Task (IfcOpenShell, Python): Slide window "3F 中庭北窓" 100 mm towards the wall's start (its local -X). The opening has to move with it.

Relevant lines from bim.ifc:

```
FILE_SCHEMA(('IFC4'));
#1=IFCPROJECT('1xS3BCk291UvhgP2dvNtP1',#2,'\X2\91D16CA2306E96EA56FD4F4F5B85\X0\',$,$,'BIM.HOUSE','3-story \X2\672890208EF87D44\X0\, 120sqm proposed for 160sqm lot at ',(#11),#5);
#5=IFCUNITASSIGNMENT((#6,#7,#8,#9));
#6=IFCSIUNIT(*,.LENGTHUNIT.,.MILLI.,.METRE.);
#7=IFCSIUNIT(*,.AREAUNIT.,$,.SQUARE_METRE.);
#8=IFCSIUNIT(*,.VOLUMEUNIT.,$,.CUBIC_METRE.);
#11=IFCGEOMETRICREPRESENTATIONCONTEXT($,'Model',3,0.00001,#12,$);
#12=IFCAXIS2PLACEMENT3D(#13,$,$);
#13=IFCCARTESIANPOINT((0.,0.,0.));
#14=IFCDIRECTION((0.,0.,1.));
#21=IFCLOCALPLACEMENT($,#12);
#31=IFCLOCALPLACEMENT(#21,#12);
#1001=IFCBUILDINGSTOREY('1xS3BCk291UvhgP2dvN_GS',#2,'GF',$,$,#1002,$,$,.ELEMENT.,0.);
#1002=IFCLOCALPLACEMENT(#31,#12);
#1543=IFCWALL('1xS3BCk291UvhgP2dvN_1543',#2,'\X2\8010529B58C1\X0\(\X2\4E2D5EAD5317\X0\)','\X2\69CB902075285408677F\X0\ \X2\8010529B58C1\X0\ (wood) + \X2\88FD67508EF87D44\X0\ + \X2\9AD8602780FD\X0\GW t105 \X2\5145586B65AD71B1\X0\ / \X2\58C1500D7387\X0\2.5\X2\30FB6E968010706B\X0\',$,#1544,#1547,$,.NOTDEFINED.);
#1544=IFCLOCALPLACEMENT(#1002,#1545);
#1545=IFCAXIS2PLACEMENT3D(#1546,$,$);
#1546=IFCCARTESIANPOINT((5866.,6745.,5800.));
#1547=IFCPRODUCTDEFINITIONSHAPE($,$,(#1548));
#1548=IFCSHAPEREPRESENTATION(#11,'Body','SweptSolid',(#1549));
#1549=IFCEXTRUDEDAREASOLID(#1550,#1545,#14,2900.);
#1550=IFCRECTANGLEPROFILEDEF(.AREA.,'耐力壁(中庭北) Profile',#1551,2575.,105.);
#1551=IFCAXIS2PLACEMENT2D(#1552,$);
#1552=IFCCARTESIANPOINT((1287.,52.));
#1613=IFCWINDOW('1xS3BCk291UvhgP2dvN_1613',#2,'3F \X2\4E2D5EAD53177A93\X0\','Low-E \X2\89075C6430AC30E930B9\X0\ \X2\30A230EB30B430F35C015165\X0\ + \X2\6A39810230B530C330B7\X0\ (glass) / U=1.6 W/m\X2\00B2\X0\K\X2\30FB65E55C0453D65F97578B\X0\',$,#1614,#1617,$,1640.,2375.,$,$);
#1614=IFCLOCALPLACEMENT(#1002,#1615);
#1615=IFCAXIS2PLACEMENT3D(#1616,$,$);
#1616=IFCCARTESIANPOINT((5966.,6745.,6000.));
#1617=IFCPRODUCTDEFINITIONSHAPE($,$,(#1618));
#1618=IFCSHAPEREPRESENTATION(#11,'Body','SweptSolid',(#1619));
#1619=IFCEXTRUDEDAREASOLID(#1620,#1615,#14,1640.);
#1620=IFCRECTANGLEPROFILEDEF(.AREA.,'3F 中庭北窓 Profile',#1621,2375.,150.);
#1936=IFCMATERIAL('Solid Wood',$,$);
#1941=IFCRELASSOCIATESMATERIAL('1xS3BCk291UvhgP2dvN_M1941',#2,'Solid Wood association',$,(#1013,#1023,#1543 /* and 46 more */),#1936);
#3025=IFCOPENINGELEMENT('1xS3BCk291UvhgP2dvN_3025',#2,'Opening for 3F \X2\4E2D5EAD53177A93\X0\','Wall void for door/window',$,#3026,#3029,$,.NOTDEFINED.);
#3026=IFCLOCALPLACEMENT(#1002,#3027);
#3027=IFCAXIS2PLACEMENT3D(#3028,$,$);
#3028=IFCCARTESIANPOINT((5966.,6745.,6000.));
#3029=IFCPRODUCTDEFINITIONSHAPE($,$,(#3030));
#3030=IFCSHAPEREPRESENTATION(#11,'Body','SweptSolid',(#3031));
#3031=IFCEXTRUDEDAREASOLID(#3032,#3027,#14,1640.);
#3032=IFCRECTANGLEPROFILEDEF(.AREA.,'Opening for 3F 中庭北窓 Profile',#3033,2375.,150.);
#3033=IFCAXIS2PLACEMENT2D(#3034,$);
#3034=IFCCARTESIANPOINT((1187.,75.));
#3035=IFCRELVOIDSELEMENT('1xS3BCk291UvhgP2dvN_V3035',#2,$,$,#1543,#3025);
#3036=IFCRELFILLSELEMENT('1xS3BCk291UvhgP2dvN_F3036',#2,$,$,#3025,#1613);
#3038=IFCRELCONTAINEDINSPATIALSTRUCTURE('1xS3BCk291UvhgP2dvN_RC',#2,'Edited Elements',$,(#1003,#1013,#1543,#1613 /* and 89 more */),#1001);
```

```python
import ifcopenshell
import ifcopenshell.api.geometry
import ifcopenshell.util.placement
import ifcopenshell.util.unit

model = ifcopenshell.open("bim.ifc")
unit_scale = ifcopenshell.util.unit.calculate_unit_scale(model)

window = model.by_id(1613)
opening = window.FillsVoids[0].RelatingOpeningElement
wall = opening.VoidsElements[0].RelatingBuildingElement

wall_matrix = ifcopenshell.util.placement.get_local_placement(wall.ObjectPlacement)
shift = wall_matrix[:3, 0] * -0.1 / unit_scale
before = ifcopenshell.util.placement.get_local_placement(window.ObjectPlacement)[:3, 3].copy()

# The window is not placed relative to its opening, so move both.
for product in (opening, window):
    matrix = ifcopenshell.util.placement.get_local_placement(product.ObjectPlacement)
    matrix[:3, 3] += shift
    ifcopenshell.api.geometry.edit_object_placement(model, product=product, matrix=matrix, is_si=False)

after = ifcopenshell.util.placement.get_local_placement(window.ObjectPlacement)[:3, 3]
print("window moved by", (after - before).round(3) + 0.0)

model.write("bim_rev.ifc")
```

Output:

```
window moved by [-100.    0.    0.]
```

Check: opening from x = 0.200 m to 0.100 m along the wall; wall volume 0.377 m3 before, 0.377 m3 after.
